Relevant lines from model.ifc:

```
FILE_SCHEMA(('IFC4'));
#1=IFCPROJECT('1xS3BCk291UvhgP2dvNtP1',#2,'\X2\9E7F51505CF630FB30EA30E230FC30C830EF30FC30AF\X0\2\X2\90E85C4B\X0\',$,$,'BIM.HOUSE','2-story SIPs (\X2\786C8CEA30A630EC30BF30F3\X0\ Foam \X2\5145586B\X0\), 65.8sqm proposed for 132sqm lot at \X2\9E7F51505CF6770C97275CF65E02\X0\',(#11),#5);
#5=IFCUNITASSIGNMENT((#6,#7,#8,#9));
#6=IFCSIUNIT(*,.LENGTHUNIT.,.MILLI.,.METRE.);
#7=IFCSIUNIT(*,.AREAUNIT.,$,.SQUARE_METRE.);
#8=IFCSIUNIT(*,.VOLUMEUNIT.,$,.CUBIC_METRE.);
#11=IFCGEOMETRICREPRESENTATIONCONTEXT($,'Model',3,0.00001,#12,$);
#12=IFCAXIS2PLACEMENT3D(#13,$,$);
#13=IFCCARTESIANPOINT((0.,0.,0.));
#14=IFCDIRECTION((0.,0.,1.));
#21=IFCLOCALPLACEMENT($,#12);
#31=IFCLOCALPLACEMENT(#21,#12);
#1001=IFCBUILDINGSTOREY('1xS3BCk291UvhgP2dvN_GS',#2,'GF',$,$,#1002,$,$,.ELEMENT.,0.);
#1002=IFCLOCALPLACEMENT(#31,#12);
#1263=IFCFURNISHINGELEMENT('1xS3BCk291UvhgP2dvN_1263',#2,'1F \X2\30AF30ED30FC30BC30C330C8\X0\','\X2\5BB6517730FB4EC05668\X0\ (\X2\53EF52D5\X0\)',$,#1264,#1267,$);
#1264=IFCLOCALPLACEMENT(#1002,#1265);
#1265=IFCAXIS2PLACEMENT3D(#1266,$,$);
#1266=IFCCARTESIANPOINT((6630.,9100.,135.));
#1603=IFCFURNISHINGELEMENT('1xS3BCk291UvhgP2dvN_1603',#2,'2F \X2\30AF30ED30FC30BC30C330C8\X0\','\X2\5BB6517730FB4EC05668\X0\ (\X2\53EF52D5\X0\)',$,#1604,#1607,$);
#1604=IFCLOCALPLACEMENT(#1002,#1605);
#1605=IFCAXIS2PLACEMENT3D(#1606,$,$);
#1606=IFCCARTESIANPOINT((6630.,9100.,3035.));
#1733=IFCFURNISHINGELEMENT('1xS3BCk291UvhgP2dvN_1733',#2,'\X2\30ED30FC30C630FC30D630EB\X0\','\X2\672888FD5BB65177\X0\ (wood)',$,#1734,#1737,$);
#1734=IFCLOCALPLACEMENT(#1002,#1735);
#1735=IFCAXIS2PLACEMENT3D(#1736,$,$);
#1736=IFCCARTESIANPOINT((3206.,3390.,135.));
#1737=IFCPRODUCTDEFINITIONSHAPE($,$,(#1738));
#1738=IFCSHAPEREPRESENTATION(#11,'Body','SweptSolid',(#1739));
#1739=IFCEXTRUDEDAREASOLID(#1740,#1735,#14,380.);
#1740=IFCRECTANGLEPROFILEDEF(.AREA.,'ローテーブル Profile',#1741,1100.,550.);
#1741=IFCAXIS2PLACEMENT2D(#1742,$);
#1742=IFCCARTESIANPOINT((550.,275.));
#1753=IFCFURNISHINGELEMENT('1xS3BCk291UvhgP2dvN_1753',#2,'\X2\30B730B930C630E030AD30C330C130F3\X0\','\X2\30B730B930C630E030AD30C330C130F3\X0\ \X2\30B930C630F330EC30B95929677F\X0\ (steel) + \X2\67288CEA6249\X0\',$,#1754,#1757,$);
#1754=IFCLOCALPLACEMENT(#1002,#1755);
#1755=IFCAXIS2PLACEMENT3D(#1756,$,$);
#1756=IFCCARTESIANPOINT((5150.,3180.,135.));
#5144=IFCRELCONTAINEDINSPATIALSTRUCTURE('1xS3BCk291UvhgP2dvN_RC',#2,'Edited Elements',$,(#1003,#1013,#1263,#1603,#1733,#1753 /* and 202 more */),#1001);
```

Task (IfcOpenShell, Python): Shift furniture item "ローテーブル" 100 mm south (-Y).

```python
import ifcopenshell
import ifcopenshell.api.geometry
import ifcopenshell.util.placement

model = ifcopenshell.open("model.ifc")

item = model.by_guid("1xS3BCk291UvhgP2dvN_1733")
matrix = ifcopenshell.util.placement.get_local_placement(item.ObjectPlacement)
matrix[1, 3] -= 100.0
ifcopenshell.api.geometry.edit_object_placement(model, product=item, matrix=matrix, is_si=False)

print(ifcopenshell.util.placement.get_local_placement(item.ObjectPlacement).round(3) + 0.0)

model.write("model_rev.ifc")
```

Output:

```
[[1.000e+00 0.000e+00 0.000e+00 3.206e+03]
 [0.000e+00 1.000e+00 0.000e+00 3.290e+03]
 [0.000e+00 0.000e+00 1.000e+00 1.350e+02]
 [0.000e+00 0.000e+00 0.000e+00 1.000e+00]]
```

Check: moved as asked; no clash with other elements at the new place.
